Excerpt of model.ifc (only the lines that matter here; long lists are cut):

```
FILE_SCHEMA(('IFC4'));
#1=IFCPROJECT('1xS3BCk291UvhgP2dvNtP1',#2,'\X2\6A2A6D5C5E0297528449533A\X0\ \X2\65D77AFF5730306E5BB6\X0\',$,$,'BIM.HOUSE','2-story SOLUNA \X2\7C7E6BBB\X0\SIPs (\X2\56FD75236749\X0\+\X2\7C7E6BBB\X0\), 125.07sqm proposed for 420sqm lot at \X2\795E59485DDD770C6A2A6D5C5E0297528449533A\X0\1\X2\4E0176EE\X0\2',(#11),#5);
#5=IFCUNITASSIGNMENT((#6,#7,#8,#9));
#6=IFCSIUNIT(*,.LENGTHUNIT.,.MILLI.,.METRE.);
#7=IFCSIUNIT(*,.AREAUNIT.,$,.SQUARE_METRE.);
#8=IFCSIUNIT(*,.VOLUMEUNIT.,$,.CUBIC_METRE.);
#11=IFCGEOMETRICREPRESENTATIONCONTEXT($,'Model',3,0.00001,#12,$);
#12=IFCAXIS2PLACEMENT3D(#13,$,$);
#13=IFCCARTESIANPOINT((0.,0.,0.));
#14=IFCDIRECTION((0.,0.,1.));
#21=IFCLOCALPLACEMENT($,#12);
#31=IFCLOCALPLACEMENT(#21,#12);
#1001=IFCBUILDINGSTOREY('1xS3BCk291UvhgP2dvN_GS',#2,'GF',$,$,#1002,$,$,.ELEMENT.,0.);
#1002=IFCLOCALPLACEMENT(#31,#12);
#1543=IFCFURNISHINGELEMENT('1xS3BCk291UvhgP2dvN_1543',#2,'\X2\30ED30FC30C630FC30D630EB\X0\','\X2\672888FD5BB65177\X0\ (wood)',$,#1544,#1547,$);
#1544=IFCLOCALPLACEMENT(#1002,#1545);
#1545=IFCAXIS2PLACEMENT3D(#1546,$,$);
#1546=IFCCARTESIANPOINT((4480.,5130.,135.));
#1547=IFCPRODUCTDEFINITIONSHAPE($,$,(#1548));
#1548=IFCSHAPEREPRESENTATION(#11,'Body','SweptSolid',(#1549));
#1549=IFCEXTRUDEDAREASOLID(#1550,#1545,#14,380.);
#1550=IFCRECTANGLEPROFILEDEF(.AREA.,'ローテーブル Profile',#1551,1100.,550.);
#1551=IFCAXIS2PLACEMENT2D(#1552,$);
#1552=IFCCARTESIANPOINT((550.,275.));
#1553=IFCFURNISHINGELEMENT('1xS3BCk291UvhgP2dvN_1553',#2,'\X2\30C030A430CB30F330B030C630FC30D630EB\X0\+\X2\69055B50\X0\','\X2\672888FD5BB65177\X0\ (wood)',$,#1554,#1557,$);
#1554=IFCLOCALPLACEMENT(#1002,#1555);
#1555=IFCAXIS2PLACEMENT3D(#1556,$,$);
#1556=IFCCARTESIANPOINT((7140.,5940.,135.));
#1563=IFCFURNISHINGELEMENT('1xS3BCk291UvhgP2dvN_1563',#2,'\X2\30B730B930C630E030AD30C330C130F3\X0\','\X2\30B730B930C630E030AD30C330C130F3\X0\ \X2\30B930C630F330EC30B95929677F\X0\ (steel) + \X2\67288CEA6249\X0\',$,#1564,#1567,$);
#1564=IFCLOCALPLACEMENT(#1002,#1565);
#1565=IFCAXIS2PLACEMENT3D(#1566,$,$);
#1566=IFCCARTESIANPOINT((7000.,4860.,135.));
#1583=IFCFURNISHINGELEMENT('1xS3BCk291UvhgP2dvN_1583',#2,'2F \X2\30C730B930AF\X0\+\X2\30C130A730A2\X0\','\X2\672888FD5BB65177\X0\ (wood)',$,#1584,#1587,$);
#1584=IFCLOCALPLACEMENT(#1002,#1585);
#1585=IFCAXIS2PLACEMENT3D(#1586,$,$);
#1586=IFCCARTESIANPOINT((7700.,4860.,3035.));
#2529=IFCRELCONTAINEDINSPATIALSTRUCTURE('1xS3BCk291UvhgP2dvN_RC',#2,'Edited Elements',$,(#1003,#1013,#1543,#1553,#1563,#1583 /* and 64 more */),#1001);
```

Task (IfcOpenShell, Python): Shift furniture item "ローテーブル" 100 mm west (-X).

```python
import ifcopenshell
import ifcopenshell.api.geometry
import ifcopenshell.util.placement
import ifcopenshell.util.unit

model = ifcopenshell.open("model.ifc")
unit_scale = ifcopenshell.util.unit.calculate_unit_scale(model)

item = model.by_guid("1xS3BCk291UvhgP2dvN_1543")
matrix = ifcopenshell.util.placement.get_local_placement(item.ObjectPlacement)
matrix[0, 3] -= 0.1 / unit_scale
ifcopenshell.api.geometry.edit_object_placement(model, product=item, matrix=matrix, is_si=False)

print(ifcopenshell.util.placement.get_local_placement(item.ObjectPlacement).round(3) + 0.0)

model.write("model_rev.ifc")
```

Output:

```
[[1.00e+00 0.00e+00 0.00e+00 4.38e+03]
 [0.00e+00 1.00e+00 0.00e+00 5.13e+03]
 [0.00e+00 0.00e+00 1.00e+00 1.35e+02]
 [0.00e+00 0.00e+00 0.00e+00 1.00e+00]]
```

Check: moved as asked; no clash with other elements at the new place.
